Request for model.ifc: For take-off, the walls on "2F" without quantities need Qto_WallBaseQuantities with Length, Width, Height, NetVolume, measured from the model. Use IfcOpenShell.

First a look at what the model holds.

```python
import ifcopenshell
import ifcopenshell.util.element
import ifcopenshell.util.unit

model = ifcopenshell.open("model.ifc")
print(model.schema)
for unit_type in ("LENGTHUNIT", "AREAUNIT", "VOLUMEUNIT"):
    print(unit_type, ifcopenshell.util.unit.calculate_unit_scale(model, unit_type))
storey = next(s for s in model.by_type("IfcBuildingStorey") if s.Name == "2F")
walls = [e for e in ifcopenshell.util.element.get_decomposition(storey) if e.is_a("IfcWall")]
for e in sorted(walls, key=lambda e: e.id()):
    print(e.id(), e.is_a(), e.Name, list(ifcopenshell.util.element.get_psets(e, qtos_only=True)), sep=" | ")
```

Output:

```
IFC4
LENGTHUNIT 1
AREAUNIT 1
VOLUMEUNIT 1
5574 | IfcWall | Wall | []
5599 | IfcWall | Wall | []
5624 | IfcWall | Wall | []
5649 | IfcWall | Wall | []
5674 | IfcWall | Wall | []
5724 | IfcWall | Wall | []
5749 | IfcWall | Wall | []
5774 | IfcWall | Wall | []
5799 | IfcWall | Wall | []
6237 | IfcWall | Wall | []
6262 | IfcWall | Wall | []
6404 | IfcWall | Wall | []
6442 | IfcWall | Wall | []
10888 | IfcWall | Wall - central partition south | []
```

```python
import ifcopenshell
import ifcopenshell.api.pset
import ifcopenshell.geom
import ifcopenshell.util.element
import ifcopenshell.util.shape
import ifcopenshell.util.unit

model = ifcopenshell.open("model.ifc")
unit_scale = ifcopenshell.util.unit.calculate_unit_scale(model)
volume_scale = ifcopenshell.util.unit.calculate_unit_scale(model, "VOLUMEUNIT")
settings = ifcopenshell.geom.settings()

storey = next(s for s in model.by_type("IfcBuildingStorey") if s.Name == "2F")
walls = [e for e in ifcopenshell.util.element.get_decomposition(storey) if e.is_a("IfcWall")]

for e in sorted(walls, key=lambda e: e.id()):
    if ifcopenshell.util.element.get_psets(e, qtos_only=True, should_inherit=False):
        continue
    # Geometry comes back in metres, in the element's own axes.
    shape = ifcopenshell.geom.create_shape(settings, e)
    values = {
        "Length": ifcopenshell.util.shape.get_x(shape.geometry) / unit_scale,
        "Width": ifcopenshell.util.shape.get_y(shape.geometry) / unit_scale,
        "Height": ifcopenshell.util.shape.get_z(shape.geometry) / unit_scale,
        "NetVolume": ifcopenshell.util.shape.get_volume(shape.geometry) / volume_scale,
    }
    qto = ifcopenshell.api.pset.add_qto(model, product=e, name="Qto_WallBaseQuantities")
    ifcopenshell.api.pset.edit_qto(model, qto=qto, properties=values)
    print(e.id(), {k: round(v, 3) for k, v in values.items()})

model.write("model-out.ifc")
```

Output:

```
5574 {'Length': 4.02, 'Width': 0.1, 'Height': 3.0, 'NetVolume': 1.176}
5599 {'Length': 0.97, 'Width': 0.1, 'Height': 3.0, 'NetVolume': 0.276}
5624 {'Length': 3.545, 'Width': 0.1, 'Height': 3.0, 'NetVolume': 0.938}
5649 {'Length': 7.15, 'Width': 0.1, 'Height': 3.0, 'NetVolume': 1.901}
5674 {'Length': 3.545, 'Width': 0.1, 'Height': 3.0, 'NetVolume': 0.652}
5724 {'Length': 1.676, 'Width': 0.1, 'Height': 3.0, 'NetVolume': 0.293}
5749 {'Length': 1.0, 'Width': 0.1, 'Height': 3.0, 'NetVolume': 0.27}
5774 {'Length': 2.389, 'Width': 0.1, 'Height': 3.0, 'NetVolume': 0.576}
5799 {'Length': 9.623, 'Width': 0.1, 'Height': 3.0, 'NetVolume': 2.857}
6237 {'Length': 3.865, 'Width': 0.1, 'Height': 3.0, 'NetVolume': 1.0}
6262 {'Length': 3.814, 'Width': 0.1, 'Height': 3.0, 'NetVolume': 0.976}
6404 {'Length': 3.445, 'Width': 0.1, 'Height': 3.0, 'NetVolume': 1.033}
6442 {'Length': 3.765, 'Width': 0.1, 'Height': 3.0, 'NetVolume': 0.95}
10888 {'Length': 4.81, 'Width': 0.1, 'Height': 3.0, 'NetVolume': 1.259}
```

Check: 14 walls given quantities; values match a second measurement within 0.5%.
